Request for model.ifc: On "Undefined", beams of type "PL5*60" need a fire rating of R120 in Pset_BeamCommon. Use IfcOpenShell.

First a look at what the model holds.

```python
import ifcopenshell
import ifcopenshell.util.element

model = ifcopenshell.open("model.ifc")
print(model.schema)
storey = next(s for s in model.by_type("IfcBuildingStorey") if s.Name == "Undefined")
beams = [e for e in ifcopenshell.util.element.get_decomposition(storey) if e.is_a("IfcBeam")]
seen = {}
for e in beams:
    element_type = ifcopenshell.util.element.get_type(e)
    key = (element_type.Name if element_type != e and element_type else None, ifcopenshell.util.element.get_pset(e, "Pset_BeamCommon", "FireRating"))
    seen[key] = seen.get(key, 0) + 1
for (name, value), count in sorted(seen.items(), key=str):
    print(count, "x", name, "|", value)
```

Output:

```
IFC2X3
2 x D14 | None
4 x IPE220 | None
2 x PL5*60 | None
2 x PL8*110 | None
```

```python
import ifcopenshell
import ifcopenshell.api.pset
import ifcopenshell.util.element

model = ifcopenshell.open("model.ifc")

storey = next(s for s in model.by_type("IfcBuildingStorey") if s.Name == "Undefined")
beams = [e for e in ifcopenshell.util.element.get_decomposition(storey) if e.is_a("IfcBeam")]

count = 0
for e in beams:
    element_type = ifcopenshell.util.element.get_type(e)
    if element_type in (None, e) or element_type.Name != "PL5*60":
        continue
    found = ifcopenshell.util.element.get_pset(e, "Pset_BeamCommon", should_inherit=False)
    if found:
        pset = model.by_id(found["id"])
        if len(ifcopenshell.util.element.get_elements_by_pset(pset)) > 1:
            pset = ifcopenshell.api.pset.unshare_pset(model, products=[e], pset=pset)[0]
    else:
        pset = ifcopenshell.api.pset.add_pset(model, product=e, name="Pset_BeamCommon")
    ifcopenshell.api.pset.edit_pset(model, pset=pset, properties={"FireRating": "R120"})
    count += 1

print(count, "beams updated")

model.write("model_edited.ifc")
```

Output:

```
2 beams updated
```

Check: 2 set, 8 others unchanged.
